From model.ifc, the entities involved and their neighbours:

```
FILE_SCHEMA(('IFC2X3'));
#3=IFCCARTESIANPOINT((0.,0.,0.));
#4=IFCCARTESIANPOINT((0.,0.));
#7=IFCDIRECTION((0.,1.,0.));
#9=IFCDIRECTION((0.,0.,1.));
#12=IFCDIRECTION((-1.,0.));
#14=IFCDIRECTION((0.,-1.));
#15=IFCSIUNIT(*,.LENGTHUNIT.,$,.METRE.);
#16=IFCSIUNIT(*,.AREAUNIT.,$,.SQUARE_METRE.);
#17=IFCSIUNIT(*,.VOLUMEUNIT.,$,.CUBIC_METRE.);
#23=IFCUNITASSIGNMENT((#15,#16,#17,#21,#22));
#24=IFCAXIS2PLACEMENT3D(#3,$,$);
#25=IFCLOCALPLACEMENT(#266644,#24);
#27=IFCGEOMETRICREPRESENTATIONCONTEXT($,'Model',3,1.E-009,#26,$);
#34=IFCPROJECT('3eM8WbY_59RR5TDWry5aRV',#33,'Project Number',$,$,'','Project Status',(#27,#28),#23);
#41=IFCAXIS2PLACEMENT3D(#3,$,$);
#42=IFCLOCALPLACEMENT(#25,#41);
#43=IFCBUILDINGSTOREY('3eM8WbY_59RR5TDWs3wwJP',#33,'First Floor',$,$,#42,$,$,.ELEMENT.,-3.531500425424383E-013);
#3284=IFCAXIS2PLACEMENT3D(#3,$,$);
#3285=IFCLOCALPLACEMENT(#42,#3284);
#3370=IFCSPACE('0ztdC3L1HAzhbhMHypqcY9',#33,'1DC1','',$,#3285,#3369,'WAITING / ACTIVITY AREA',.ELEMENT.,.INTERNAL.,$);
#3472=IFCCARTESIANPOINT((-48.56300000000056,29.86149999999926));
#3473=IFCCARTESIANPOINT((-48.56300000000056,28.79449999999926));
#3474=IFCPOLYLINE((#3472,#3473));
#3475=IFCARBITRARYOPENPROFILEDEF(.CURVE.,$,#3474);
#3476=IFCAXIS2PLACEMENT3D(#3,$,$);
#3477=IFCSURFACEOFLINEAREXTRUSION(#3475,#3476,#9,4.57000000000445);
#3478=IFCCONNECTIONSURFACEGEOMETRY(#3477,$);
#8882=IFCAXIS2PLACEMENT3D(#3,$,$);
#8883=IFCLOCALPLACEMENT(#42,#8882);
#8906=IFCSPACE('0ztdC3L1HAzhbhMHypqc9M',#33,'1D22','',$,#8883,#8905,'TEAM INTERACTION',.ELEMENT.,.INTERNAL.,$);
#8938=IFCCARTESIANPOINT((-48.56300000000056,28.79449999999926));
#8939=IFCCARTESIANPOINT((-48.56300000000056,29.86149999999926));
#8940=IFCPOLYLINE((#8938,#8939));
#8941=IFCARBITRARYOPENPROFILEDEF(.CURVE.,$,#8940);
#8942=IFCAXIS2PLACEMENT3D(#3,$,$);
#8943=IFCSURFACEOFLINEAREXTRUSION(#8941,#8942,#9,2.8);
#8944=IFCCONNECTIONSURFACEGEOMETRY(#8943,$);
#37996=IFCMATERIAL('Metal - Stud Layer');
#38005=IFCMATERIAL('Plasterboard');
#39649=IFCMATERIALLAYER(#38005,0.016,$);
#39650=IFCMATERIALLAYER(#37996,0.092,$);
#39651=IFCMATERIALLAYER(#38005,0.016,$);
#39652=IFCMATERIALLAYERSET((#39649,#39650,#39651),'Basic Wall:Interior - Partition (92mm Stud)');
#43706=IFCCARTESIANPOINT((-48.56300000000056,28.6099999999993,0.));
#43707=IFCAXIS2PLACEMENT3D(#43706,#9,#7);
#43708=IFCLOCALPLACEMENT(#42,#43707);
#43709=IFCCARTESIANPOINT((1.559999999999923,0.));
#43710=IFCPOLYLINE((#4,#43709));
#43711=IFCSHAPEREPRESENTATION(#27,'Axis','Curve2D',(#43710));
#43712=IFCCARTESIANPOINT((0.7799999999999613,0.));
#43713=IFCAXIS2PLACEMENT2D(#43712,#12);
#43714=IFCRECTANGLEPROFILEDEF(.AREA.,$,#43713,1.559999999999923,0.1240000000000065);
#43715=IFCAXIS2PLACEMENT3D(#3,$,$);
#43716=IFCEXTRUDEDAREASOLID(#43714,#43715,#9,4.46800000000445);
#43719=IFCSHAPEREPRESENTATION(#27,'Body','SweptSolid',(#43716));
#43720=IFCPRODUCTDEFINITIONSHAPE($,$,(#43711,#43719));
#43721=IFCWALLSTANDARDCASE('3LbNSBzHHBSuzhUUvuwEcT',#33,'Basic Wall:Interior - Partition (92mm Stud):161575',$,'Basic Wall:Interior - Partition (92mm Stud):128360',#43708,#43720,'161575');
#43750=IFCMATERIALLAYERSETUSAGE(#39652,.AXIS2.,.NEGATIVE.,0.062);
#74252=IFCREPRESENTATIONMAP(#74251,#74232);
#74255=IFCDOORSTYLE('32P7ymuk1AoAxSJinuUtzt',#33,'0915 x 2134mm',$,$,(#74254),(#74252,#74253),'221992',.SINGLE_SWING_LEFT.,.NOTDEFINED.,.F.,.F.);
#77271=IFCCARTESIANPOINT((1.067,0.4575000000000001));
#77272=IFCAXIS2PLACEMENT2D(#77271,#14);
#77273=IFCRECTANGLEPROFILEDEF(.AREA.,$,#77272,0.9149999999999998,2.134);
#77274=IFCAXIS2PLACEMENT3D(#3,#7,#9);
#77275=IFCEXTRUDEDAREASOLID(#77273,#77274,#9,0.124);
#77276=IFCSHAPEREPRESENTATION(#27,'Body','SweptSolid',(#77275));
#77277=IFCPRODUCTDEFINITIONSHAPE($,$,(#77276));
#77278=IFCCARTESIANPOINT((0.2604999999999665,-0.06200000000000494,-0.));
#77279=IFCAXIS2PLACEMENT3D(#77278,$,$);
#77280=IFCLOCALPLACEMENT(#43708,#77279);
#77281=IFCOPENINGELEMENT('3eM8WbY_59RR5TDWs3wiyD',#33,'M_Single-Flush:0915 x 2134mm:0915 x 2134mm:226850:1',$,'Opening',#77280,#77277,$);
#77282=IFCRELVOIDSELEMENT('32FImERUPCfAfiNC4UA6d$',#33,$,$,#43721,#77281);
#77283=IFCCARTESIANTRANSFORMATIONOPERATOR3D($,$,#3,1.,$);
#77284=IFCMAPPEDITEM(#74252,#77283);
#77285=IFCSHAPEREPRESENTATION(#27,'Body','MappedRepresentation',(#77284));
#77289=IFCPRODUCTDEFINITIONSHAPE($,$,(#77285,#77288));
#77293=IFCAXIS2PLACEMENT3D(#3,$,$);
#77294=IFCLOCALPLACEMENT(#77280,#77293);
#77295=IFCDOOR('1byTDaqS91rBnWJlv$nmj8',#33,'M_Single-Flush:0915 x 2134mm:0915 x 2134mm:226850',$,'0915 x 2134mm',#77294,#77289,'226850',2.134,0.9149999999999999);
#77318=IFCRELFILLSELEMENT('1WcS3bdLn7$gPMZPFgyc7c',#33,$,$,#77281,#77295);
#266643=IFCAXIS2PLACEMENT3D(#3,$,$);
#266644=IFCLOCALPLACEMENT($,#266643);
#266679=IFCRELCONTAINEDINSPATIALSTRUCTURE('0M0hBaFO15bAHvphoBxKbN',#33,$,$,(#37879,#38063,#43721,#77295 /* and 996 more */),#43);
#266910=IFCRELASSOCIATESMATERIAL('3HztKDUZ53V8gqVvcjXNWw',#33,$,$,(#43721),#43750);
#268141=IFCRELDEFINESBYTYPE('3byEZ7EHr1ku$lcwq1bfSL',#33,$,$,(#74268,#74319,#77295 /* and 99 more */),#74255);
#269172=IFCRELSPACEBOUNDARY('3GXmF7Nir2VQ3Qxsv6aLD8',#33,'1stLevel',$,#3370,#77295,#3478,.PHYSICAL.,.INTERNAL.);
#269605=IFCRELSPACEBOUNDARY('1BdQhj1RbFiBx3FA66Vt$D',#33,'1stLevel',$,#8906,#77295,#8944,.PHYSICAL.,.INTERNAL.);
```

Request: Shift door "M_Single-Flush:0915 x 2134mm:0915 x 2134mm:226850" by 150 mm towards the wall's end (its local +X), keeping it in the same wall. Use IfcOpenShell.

```python
import numpy as np
import ifcopenshell
import ifcopenshell.api.geometry
import ifcopenshell.util.placement

model = ifcopenshell.open("model.ifc")

door = model.by_id(77295)
opening = door.FillsVoids[0].RelatingOpeningElement
wall = opening.VoidsElements[0].RelatingBuildingElement

wall_matrix = ifcopenshell.util.placement.get_local_placement(wall.ObjectPlacement)
shift = wall_matrix[:3, 0] * 0.15
before = ifcopenshell.util.placement.get_local_placement(door.ObjectPlacement)[:3, 3].copy()

# The door is placed relative to its opening, so it follows when the opening moves.
matrix = ifcopenshell.util.placement.get_local_placement(opening.ObjectPlacement)
matrix[:3, 3] += shift
ifcopenshell.api.geometry.edit_object_placement(
    model, product=opening, matrix=matrix, is_si=False, should_transform_children=True
)

# Space boundary surfaces are stored in each space's coordinates; move them too.
for rel in door.ProvidesBoundaries:
    if not rel.ConnectionGeometry:
        continue
    surface = rel.ConnectionGeometry.SurfaceOnRelatingElement
    space_matrix = ifcopenshell.util.placement.get_local_placement(rel.RelatingSpace.ObjectPlacement)
    point = np.array(surface.Position.Location.Coordinates) + space_matrix[:3, :3].T @ shift
    surface.Position = model.createIfcAxis2Placement3D(
        model.createIfcCartesianPoint(point.tolist()), surface.Position.Axis, surface.Position.RefDirection
    )

after = ifcopenshell.util.placement.get_local_placement(door.ObjectPlacement)[:3, 3]
print("door moved by", (after - before).round(3) + 0.0)

model.write("model_edited.ifc")
```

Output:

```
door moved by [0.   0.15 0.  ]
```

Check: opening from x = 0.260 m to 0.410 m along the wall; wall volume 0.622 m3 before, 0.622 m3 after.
